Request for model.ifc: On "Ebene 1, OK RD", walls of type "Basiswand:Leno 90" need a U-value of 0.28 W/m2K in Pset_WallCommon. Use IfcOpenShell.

First a look at what the model holds.

```python
import ifcopenshell
import ifcopenshell.util.element

model = ifcopenshell.open("model.ifc")
print(model.schema)
storey = next(s for s in model.by_type("IfcBuildingStorey") if s.Name == "Ebene 1, OK RD")
walls = [e for e in ifcopenshell.util.element.get_decomposition(storey) if e.is_a("IfcWall")]
seen = {}
for e in walls:
    element_type = ifcopenshell.util.element.get_type(e)
    key = (element_type.Name if element_type != e and element_type else None, ifcopenshell.util.element.get_pset(e, "Pset_WallCommon", "ThermalTransmittance"))
    seen[key] = seen.get(key, 0) + 1
for (name, value), count in sorted(seen.items(), key=str):
    print(count, "x", name, "|", value)
```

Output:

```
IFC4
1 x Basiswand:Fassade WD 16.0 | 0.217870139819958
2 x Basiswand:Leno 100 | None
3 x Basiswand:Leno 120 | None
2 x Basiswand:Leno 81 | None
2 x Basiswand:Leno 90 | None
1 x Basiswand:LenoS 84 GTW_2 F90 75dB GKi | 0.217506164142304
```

```python
import ifcopenshell
import ifcopenshell.api.pset
import ifcopenshell.util.element

model = ifcopenshell.open("model.ifc")

storey = next(s for s in model.by_type("IfcBuildingStorey") if s.Name == "Ebene 1, OK RD")
walls = [e for e in ifcopenshell.util.element.get_decomposition(storey) if e.is_a("IfcWall")]

count = 0
for e in walls:
    element_type = ifcopenshell.util.element.get_type(e)
    if element_type in (None, e) or element_type.Name != "Basiswand:Leno 90":
        continue
    # add_pset returns the element's existing set when there is one.
    pset = ifcopenshell.api.pset.add_pset(model, product=e, name="Pset_WallCommon")
    ifcopenshell.api.pset.edit_pset(model, pset=pset, properties={"ThermalTransmittance": 0.28})
    count += 1

print(count, "walls updated")

model.write("model_v2.ifc")
```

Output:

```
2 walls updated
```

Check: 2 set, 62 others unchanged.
